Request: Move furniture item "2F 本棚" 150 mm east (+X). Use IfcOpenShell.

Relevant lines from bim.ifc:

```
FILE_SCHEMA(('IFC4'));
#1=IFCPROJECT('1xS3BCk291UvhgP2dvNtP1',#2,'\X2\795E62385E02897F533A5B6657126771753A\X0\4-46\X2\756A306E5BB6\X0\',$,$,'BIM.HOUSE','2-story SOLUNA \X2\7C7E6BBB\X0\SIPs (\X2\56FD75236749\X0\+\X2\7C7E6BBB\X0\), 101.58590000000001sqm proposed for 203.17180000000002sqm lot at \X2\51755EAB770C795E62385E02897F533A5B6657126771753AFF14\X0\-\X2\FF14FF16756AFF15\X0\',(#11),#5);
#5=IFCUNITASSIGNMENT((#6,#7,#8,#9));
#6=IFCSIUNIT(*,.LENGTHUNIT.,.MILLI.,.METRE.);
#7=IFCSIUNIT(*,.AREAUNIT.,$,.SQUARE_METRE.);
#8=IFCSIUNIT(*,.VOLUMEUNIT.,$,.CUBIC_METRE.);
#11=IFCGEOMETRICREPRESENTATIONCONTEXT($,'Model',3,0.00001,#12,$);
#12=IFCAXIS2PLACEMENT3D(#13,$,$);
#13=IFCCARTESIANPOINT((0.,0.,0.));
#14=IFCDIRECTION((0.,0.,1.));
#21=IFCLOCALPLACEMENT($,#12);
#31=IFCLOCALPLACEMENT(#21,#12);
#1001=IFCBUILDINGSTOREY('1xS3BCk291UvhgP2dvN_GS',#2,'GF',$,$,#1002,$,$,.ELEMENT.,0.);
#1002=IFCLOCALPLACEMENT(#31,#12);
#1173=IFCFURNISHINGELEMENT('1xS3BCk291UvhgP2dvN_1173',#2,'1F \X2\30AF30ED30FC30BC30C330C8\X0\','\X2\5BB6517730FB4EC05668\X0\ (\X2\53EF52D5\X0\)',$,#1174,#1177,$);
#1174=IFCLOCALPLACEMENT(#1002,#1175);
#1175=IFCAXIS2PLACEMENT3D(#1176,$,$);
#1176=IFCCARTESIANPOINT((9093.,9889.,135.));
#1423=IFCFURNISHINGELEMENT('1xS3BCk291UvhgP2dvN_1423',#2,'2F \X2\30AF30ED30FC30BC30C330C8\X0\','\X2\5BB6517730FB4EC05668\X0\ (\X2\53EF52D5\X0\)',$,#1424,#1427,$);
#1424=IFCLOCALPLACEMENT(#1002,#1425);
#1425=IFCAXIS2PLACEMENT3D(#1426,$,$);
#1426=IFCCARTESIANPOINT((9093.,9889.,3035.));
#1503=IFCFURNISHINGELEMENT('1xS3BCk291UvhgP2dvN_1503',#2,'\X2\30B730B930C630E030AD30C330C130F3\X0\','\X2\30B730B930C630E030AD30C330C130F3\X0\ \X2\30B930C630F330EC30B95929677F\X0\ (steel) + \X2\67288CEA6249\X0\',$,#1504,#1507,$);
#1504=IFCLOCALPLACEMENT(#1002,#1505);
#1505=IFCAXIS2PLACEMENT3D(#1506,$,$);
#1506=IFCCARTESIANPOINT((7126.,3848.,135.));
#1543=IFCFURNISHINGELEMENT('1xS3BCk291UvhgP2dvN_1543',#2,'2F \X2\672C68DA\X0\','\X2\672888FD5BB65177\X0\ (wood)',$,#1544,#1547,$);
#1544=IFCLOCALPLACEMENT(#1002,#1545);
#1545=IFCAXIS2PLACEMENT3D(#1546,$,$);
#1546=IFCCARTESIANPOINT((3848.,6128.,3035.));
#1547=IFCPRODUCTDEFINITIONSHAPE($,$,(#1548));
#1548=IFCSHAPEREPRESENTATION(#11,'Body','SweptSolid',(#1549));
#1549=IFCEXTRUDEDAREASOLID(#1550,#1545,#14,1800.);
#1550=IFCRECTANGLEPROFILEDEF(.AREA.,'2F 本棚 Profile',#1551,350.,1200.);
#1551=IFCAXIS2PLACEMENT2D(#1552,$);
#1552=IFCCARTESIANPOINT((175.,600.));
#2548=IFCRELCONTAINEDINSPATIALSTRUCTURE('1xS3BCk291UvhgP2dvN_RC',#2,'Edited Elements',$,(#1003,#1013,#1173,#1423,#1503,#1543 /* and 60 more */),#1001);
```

```python
import ifcopenshell
import ifcopenshell.api.geometry
import ifcopenshell.util.placement
import ifcopenshell.util.unit

model = ifcopenshell.open("bim.ifc")
unit_scale = ifcopenshell.util.unit.calculate_unit_scale(model)

item = model.by_guid("1xS3BCk291UvhgP2dvN_1543")
matrix = ifcopenshell.util.placement.get_local_placement(item.ObjectPlacement)
matrix[0, 3] += 0.15 / unit_scale
ifcopenshell.api.geometry.edit_object_placement(model, product=item, matrix=matrix, is_si=False)

print(ifcopenshell.util.placement.get_local_placement(item.ObjectPlacement).round(3) + 0.0)

model.write("bim_v2.ifc")
```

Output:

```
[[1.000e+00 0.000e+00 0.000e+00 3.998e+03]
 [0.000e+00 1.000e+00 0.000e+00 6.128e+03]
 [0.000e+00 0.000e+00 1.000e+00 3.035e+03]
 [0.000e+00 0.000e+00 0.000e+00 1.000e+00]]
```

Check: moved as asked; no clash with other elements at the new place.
